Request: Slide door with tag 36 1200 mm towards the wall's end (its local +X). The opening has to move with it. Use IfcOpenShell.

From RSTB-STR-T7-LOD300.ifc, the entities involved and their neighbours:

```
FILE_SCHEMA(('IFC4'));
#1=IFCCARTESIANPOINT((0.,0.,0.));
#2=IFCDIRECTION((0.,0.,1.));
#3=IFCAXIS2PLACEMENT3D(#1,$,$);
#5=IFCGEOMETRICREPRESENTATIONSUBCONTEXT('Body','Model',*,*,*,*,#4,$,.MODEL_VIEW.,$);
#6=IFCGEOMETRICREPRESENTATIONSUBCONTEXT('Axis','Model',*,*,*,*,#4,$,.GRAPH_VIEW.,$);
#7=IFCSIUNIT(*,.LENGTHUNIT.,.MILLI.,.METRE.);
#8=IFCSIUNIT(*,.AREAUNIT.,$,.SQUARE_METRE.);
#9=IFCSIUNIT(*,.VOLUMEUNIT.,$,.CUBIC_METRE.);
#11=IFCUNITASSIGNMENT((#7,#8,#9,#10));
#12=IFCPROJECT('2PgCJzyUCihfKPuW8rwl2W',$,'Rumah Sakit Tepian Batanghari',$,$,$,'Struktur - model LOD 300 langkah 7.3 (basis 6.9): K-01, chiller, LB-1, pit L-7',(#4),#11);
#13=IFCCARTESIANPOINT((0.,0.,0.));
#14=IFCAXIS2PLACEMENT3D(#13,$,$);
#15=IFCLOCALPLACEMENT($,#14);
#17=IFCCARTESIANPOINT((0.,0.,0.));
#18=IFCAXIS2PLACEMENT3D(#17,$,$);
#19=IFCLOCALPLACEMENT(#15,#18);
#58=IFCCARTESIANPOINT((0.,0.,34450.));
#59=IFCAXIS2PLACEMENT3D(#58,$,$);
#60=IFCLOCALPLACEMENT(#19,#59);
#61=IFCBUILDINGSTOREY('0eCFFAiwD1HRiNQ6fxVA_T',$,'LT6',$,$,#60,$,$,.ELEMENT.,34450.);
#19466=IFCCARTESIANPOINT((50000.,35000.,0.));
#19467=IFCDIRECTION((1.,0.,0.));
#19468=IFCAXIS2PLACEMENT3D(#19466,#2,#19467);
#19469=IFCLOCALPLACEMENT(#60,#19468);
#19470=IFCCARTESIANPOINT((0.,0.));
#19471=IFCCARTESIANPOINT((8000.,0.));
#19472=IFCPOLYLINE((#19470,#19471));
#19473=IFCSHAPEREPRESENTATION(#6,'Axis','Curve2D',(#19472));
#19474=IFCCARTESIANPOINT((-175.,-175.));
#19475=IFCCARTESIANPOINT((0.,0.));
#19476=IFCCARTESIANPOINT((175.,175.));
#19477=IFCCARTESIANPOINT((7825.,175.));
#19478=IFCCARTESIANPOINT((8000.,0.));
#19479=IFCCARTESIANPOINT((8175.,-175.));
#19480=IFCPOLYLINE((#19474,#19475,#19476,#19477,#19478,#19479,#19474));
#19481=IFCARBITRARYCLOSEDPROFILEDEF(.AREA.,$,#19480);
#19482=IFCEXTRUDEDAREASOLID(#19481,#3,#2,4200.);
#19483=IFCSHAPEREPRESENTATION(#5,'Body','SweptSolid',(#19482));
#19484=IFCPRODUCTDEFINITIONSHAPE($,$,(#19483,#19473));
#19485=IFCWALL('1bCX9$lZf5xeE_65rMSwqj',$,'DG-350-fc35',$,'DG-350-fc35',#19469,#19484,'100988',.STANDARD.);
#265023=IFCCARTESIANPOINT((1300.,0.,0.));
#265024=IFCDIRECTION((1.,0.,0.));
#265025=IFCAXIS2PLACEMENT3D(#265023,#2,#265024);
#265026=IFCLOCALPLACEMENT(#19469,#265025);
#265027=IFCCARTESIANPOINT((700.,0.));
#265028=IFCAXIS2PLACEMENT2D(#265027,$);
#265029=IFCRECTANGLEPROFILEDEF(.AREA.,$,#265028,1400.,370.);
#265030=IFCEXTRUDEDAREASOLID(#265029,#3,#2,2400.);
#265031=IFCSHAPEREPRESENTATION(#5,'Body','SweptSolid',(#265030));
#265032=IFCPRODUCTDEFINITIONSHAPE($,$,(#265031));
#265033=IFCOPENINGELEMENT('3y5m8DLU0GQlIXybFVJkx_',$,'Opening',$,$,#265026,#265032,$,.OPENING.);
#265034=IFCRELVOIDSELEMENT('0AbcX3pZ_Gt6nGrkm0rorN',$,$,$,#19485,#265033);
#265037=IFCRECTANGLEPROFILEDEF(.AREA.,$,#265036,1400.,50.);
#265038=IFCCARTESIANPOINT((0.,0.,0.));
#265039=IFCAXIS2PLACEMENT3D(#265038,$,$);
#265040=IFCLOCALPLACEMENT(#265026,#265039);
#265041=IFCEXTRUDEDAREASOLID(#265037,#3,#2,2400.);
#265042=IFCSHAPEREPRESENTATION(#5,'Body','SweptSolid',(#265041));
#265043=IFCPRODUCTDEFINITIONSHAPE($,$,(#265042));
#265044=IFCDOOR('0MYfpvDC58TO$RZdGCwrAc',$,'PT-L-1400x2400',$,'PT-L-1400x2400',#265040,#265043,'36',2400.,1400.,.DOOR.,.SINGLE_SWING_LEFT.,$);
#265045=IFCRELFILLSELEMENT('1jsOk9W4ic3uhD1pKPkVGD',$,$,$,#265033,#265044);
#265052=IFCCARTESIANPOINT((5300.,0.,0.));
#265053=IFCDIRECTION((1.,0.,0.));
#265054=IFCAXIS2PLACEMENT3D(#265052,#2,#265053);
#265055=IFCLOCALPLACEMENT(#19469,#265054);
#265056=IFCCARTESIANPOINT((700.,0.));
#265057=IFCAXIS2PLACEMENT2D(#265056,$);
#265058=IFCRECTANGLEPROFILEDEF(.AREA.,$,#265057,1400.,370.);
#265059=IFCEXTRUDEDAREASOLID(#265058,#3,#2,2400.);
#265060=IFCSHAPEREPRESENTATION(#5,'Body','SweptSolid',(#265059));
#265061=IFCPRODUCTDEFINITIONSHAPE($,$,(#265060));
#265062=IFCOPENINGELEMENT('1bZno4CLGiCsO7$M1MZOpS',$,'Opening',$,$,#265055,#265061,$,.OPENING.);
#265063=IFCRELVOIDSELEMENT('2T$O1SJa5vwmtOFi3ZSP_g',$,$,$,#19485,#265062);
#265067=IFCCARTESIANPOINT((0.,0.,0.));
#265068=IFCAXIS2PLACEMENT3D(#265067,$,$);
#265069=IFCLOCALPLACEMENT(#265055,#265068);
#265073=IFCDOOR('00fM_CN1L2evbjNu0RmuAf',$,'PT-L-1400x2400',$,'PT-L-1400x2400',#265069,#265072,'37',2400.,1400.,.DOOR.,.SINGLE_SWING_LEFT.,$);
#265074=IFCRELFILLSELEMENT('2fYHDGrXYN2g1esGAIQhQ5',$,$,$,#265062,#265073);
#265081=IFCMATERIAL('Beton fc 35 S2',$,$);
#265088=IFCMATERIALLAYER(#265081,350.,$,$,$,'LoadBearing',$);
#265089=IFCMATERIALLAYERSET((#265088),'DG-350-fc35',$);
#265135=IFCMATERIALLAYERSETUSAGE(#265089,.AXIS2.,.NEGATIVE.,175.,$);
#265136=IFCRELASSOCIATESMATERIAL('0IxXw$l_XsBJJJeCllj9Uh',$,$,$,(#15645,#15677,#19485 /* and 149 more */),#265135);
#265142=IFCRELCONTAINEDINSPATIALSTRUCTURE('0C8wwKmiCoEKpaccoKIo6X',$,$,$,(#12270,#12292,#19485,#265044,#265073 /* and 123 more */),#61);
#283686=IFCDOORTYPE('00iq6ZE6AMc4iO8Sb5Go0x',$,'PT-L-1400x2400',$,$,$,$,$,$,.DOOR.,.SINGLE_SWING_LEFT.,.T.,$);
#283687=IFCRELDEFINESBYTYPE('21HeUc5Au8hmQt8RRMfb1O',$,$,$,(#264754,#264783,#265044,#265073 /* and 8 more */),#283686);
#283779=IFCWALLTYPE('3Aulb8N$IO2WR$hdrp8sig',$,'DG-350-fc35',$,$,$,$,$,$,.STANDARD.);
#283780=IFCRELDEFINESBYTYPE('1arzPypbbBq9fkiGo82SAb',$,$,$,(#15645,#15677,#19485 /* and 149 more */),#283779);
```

```python
import ifcopenshell
import ifcopenshell.api.geometry
import ifcopenshell.util.placement

model = ifcopenshell.open("RSTB-STR-T7-LOD300.ifc")

door = model.by_guid("0MYfpvDC58TO$RZdGCwrAc")
opening = door.FillsVoids[0].RelatingOpeningElement
wall = opening.VoidsElements[0].RelatingBuildingElement

wall_matrix = ifcopenshell.util.placement.get_local_placement(wall.ObjectPlacement)
shift = wall_matrix[:3, 0] * 1200.0
before = ifcopenshell.util.placement.get_local_placement(door.ObjectPlacement)[:3, 3].copy()

# The door is placed relative to its opening, so it follows when the opening moves.
matrix = ifcopenshell.util.placement.get_local_placement(opening.ObjectPlacement)
matrix[:3, 3] += shift
ifcopenshell.api.geometry.edit_object_placement(
    model, product=opening, matrix=matrix, is_si=False, should_transform_children=True
)

after = ifcopenshell.util.placement.get_local_placement(door.ObjectPlacement)[:3, 3]
print("door moved by", (after - before).round(3) + 0.0)

model.write("RSTB-STR-T7-LOD300-out.ifc")
```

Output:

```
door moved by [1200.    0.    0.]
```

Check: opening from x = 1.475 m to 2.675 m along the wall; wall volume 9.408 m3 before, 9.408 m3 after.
